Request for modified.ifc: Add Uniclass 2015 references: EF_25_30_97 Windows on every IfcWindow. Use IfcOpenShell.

First a look at what the model holds.

```python
import ifcopenshell

model = ifcopenshell.open("modified.ifc")
print(model.schema)
print("classifications:", [c.Name for c in model.by_type("IfcClassification")])
for ifc_class in ("IfcDoor", "IfcRoof", "IfcStair", "IfcWall", "IfcWindow"):
    print(ifc_class, len(model.by_type(ifc_class)))
```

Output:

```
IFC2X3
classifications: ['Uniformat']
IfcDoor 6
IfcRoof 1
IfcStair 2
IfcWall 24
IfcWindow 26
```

```python
import ifcopenshell
import ifcopenshell.api.classification

model = ifcopenshell.open("modified.ifc")

# IFC2X3 requires Source and Edition and has no link from the project to the system.
system = model.create_entity("IfcClassification", Source="NBS", Edition="2015", Name="Uniclass 2015")

codes = {
    "IfcWindow": ("EF_25_30_97", "Windows"),
}
for ifc_class, (code, name) in codes.items():
    products = model.by_type(ifc_class)
    ifcopenshell.api.classification.add_reference(
        model, products=products, classification=system, identification=code, name=name
    )
    print(code, len(products))

model.write("modified_rev.ifc")
```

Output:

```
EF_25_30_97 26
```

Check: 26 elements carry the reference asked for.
